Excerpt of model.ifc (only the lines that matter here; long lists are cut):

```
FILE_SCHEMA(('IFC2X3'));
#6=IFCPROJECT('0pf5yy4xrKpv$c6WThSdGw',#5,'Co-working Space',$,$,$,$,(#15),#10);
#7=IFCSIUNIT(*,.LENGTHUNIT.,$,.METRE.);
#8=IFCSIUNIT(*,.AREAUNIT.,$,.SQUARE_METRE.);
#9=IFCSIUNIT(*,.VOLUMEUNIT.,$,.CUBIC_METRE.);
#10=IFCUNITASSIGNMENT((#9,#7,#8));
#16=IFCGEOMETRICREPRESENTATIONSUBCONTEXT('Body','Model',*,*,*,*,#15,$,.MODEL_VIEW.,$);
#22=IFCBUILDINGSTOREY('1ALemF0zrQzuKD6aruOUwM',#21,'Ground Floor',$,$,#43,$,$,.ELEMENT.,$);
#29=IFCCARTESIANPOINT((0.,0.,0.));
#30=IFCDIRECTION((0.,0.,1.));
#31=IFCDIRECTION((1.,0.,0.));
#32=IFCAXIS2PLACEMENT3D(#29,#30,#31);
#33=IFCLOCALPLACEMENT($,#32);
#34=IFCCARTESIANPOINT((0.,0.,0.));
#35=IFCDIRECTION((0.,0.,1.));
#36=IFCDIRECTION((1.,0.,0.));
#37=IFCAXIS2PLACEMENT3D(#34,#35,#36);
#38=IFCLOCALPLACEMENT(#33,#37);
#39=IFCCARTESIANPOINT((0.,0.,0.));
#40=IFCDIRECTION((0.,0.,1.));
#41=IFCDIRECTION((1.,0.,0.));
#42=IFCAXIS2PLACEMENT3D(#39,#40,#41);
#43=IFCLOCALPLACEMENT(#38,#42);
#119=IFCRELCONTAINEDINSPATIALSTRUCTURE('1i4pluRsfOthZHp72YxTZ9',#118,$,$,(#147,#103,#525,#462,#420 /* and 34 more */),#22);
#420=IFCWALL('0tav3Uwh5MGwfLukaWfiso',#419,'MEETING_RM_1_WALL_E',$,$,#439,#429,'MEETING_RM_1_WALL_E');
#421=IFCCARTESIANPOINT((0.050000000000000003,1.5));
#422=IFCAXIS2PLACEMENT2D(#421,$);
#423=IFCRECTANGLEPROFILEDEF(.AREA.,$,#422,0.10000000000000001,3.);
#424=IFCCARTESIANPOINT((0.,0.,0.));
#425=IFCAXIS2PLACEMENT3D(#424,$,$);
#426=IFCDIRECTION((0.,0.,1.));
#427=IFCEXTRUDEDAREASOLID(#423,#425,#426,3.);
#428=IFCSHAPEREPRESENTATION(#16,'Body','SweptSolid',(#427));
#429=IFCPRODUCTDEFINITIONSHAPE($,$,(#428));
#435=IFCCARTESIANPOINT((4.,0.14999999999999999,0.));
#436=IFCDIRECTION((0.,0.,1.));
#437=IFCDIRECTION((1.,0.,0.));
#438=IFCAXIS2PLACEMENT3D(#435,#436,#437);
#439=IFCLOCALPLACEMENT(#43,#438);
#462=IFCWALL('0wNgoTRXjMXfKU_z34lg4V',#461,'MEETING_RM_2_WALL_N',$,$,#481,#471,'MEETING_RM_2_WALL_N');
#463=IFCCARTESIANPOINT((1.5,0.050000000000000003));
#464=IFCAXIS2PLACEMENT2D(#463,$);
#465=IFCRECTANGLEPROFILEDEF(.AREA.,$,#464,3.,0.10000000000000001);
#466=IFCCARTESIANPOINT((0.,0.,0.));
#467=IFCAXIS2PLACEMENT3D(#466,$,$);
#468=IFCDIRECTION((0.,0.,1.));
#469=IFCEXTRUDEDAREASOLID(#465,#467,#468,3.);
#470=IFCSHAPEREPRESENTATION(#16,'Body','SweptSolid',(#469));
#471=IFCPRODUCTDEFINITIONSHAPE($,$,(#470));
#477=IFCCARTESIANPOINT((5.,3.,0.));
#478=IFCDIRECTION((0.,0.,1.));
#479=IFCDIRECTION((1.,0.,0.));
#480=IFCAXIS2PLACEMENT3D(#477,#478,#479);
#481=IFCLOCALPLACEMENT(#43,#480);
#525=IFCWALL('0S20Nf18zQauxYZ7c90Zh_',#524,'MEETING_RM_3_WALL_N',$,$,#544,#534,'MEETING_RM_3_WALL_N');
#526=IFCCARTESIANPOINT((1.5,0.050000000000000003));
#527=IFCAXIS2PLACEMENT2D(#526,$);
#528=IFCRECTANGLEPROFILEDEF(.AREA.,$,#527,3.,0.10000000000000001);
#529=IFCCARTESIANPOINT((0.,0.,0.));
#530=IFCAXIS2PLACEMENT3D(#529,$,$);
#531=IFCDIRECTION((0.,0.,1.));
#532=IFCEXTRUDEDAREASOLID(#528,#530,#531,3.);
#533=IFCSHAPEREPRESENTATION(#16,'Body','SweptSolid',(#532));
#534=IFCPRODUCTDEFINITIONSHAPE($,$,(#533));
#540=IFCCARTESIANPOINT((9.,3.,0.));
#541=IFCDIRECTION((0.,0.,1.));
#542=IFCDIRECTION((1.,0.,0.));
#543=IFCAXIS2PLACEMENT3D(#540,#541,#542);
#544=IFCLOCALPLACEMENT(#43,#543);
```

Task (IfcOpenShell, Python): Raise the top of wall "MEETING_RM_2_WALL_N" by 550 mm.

```python
import ifcopenshell
import ifcopenshell.geom
import ifcopenshell.util.representation
import ifcopenshell.util.shape

model = ifcopenshell.open("model.ifc")
settings = ifcopenshell.geom.settings()


def volume(element):
    """Net volume in cubic metres, openings subtracted."""
    shape = ifcopenshell.geom.create_shape(settings, element)
    return ifcopenshell.util.shape.get_volume(shape.geometry)


wall = model.by_id(462)
before = volume(wall)

body = ifcopenshell.util.representation.get_representation(wall, "Model", "Body")
solid = body.Items[0]
old_height = solid.Depth
solid.Depth += 0.55
after = volume(wall)

print(f"height {old_height:g} -> {solid.Depth:g}, volume {before:.3f} -> {after:.3f} m3")

model.write("model_edited.ifc")
```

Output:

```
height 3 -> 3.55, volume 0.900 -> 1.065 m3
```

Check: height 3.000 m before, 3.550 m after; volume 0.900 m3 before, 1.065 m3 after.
